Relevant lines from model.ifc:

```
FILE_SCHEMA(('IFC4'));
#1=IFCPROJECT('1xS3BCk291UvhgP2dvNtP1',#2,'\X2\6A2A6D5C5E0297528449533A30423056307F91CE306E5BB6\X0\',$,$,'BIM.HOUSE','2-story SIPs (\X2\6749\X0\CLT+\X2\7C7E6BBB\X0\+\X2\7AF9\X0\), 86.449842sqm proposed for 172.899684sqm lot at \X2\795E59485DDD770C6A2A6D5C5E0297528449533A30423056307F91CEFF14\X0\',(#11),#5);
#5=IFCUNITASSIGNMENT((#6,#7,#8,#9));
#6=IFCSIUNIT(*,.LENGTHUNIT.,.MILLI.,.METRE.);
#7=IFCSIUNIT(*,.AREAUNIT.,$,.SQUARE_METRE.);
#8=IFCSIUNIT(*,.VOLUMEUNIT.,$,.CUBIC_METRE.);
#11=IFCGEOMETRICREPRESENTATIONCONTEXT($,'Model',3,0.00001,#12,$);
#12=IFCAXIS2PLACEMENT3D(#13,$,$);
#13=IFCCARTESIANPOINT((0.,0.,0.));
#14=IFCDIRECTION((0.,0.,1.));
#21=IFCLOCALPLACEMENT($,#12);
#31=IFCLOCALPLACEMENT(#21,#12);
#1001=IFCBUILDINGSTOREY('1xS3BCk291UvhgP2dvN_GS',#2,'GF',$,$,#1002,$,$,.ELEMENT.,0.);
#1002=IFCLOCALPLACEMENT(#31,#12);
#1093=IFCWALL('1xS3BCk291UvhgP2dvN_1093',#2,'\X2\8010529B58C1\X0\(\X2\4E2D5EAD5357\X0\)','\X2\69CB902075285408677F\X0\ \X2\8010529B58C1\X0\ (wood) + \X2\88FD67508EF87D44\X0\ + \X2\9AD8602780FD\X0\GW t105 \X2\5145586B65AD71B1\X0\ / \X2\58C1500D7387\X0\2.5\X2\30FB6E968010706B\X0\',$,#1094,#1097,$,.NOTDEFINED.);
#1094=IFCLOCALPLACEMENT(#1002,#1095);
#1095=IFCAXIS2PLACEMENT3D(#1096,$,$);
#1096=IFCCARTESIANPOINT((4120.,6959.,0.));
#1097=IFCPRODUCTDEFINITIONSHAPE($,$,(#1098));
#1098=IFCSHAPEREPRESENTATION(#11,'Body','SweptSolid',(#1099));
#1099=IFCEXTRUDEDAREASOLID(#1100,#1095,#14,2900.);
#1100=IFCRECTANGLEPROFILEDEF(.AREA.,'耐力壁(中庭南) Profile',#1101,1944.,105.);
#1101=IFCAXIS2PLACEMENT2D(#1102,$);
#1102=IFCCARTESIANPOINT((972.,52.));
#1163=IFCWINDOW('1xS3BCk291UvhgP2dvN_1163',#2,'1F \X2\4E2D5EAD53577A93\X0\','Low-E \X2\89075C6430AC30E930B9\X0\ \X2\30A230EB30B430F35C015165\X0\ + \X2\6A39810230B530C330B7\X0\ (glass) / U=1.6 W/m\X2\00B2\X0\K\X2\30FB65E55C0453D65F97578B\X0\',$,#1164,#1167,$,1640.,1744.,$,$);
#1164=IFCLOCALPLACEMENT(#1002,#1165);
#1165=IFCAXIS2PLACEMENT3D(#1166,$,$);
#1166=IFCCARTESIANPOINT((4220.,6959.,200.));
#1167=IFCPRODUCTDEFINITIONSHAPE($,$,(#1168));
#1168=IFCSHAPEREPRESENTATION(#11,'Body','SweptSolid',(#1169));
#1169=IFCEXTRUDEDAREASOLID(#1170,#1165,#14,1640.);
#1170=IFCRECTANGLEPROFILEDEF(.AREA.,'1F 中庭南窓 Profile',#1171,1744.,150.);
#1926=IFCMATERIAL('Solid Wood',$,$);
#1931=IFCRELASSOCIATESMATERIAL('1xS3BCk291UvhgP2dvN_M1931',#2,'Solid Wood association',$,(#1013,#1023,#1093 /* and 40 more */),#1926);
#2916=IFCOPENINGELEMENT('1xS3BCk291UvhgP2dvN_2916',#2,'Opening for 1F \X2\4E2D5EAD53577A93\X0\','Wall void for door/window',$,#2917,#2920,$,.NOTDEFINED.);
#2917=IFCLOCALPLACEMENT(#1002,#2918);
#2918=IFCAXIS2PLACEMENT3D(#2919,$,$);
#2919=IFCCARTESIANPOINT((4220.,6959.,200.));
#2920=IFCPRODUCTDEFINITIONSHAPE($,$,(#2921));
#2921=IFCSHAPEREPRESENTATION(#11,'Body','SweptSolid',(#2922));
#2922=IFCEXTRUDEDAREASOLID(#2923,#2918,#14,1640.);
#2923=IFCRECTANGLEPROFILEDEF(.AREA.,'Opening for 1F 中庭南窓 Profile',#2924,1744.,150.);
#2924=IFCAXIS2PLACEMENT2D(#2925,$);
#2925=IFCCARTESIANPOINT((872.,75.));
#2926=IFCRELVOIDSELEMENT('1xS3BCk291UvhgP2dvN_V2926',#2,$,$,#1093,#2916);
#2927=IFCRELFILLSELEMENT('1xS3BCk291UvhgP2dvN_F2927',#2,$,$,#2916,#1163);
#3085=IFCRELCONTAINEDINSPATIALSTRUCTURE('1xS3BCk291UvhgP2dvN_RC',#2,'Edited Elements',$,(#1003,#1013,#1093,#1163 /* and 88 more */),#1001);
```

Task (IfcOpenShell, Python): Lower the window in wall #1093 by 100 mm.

```python
import numpy as np
import ifcopenshell
import ifcopenshell.api.geometry
import ifcopenshell.util.placement
import ifcopenshell.util.unit

model = ifcopenshell.open("model.ifc")
unit_scale = ifcopenshell.util.unit.calculate_unit_scale(model)

window = model.by_guid("1xS3BCk291UvhgP2dvN_1163")
opening = window.FillsVoids[0].RelatingOpeningElement
dz = -0.1 / unit_scale

shift = np.array([0.0, 0.0, dz])
# The window is not placed relative to its opening, so move both.
for product in (opening, window):
    matrix = ifcopenshell.util.placement.get_local_placement(product.ObjectPlacement)
    matrix[:3, 3] += shift
    ifcopenshell.api.geometry.edit_object_placement(model, product=product, matrix=matrix, is_si=False)

print(f"moved by {dz * unit_scale:+.3f} m")

model.write("model_edited.ifc")
```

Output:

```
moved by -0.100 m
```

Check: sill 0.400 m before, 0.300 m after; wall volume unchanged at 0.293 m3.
